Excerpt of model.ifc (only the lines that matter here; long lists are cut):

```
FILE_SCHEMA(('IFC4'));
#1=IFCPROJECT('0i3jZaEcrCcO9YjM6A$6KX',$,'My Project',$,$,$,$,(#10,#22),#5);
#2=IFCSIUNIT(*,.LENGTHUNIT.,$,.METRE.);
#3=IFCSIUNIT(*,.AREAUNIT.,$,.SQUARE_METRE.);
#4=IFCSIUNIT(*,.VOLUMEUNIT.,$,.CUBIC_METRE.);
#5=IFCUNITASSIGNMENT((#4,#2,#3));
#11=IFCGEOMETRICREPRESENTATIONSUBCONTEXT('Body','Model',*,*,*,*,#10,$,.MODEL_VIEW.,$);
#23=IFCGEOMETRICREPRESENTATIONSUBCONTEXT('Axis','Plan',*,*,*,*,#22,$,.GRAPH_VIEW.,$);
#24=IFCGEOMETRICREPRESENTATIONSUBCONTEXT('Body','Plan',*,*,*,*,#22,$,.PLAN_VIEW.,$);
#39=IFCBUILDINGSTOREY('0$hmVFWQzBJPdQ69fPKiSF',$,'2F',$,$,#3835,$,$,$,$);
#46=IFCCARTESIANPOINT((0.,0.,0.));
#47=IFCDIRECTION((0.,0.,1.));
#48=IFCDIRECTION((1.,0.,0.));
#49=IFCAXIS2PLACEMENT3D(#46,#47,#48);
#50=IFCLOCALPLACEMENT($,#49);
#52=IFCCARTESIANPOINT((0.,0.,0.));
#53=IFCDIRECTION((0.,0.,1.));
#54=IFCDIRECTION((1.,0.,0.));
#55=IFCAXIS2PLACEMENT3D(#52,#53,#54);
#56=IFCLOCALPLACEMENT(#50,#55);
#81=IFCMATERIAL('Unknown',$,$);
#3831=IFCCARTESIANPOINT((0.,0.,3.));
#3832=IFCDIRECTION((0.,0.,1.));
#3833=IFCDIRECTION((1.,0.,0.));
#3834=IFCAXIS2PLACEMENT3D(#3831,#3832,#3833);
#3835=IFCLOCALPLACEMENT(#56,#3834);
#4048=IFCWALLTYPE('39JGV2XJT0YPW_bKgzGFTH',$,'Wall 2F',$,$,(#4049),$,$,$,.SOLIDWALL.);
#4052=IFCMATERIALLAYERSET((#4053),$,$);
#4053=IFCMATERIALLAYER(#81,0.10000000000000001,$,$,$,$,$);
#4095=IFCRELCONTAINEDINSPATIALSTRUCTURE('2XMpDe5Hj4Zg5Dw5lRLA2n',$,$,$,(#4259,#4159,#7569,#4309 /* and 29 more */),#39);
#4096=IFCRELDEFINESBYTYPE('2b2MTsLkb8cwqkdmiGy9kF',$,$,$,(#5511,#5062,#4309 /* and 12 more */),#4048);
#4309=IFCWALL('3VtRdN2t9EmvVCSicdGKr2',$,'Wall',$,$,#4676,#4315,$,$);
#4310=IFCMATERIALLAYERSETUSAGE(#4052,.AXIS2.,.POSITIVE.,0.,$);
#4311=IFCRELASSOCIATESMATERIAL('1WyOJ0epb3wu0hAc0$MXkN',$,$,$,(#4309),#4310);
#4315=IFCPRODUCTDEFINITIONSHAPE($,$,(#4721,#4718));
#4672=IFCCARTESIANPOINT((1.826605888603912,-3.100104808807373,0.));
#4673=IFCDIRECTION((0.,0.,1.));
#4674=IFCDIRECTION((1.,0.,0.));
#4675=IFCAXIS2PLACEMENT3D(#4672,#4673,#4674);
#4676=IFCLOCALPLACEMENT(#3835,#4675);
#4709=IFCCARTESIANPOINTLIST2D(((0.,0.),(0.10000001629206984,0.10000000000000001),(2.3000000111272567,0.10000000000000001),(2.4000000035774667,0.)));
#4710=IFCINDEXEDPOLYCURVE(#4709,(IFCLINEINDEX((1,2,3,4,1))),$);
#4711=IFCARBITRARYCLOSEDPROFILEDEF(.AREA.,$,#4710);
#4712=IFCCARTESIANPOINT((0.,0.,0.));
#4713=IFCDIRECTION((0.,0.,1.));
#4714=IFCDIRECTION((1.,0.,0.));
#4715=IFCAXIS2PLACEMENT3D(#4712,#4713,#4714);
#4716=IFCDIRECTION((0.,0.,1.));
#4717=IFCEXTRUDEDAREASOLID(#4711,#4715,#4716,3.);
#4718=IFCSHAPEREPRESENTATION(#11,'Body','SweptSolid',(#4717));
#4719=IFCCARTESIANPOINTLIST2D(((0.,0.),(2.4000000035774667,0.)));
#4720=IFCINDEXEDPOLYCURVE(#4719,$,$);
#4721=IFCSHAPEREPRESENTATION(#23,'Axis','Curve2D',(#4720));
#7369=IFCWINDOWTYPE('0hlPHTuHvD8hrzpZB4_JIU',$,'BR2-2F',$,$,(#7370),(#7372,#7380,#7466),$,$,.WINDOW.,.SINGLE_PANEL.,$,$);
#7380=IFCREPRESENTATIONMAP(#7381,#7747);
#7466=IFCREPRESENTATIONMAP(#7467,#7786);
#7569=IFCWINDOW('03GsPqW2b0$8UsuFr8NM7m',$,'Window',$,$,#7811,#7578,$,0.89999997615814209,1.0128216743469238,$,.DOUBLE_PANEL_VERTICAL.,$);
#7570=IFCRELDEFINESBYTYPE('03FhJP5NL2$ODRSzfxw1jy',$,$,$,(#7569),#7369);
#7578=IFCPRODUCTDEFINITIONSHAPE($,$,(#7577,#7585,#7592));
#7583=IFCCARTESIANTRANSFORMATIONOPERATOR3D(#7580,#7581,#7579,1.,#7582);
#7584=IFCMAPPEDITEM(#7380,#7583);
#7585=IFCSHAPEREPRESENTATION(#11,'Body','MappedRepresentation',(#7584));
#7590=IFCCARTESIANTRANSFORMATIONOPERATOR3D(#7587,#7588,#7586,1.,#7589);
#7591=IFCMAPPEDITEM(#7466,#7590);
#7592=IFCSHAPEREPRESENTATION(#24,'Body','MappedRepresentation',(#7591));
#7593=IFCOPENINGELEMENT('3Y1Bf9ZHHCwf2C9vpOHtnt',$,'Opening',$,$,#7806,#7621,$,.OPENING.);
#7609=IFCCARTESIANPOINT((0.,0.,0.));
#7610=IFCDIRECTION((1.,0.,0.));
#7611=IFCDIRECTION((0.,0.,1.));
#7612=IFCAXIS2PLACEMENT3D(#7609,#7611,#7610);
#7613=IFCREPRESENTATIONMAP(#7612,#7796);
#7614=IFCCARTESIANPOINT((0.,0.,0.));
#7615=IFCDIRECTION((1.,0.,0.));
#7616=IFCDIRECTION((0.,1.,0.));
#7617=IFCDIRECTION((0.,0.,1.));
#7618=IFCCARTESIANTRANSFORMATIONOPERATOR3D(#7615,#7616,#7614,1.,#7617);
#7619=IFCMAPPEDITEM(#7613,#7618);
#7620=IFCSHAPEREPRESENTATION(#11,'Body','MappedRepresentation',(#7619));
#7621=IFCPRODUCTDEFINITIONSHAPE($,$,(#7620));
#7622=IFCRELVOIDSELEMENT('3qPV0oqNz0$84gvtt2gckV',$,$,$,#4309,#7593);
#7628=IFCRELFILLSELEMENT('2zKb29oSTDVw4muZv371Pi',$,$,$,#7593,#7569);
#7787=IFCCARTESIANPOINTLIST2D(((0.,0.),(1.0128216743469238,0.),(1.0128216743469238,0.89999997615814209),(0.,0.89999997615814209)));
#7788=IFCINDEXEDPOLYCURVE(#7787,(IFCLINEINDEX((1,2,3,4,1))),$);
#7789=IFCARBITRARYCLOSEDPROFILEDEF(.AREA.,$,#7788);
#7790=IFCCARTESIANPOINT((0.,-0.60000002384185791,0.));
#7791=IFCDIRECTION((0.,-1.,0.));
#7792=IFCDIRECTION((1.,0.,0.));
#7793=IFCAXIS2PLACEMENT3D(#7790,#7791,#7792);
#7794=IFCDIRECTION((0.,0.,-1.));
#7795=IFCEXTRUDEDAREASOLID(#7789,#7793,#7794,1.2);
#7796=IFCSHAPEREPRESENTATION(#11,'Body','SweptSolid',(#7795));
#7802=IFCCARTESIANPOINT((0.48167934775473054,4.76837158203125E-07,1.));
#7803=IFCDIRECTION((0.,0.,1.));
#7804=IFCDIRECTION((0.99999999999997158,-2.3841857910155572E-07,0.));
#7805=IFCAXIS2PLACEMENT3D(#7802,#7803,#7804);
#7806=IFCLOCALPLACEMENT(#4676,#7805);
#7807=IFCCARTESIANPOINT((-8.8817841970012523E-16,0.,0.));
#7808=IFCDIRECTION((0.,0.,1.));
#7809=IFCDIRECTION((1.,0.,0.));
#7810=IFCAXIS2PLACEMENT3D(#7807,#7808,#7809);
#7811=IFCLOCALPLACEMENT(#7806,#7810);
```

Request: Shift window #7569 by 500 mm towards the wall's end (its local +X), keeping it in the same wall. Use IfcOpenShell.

```python
import ifcopenshell
import ifcopenshell.api.geometry
import ifcopenshell.util.placement
import ifcopenshell.util.unit

model = ifcopenshell.open("model.ifc")
unit_scale = ifcopenshell.util.unit.calculate_unit_scale(model)

window = model.by_guid("03GsPqW2b0$8UsuFr8NM7m")
opening = window.FillsVoids[0].RelatingOpeningElement
wall = opening.VoidsElements[0].RelatingBuildingElement

wall_matrix = ifcopenshell.util.placement.get_local_placement(wall.ObjectPlacement)
shift = wall_matrix[:3, 0] * 0.5 / unit_scale
before = ifcopenshell.util.placement.get_local_placement(window.ObjectPlacement)[:3, 3].copy()

# The window is placed relative to its opening, so it follows when the opening moves.
matrix = ifcopenshell.util.placement.get_local_placement(opening.ObjectPlacement)
matrix[:3, 3] += shift
ifcopenshell.api.geometry.edit_object_placement(
    model, product=opening, matrix=matrix, is_si=False, should_transform_children=True
)

after = ifcopenshell.util.placement.get_local_placement(window.ObjectPlacement)[:3, 3]
print("window moved by", (after - before).round(3) + 0.0)

model.write("model_v2.ifc")
```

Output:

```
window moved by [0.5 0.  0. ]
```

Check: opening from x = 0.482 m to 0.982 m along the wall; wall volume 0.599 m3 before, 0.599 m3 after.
